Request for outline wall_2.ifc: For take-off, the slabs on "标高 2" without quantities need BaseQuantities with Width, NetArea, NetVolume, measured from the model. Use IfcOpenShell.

First a look at what the model holds.

```python
import ifcopenshell
import ifcopenshell.util.element
import ifcopenshell.util.unit

model = ifcopenshell.open("outline wall_2.ifc")
print(model.schema)
for unit_type in ("LENGTHUNIT", "AREAUNIT", "VOLUMEUNIT"):
    print(unit_type, ifcopenshell.util.unit.calculate_unit_scale(model, unit_type))
storey = next(s for s in model.by_type("IfcBuildingStorey") if s.Name == "标高 2")
slabs = [e for e in ifcopenshell.util.element.get_decomposition(storey) if e.is_a("IfcSlab")]
for e in sorted(slabs, key=lambda e: e.id()):
    print(e.id(), e.is_a(), e.Name, list(ifcopenshell.util.element.get_psets(e, qtos_only=True)), sep=" | ")
```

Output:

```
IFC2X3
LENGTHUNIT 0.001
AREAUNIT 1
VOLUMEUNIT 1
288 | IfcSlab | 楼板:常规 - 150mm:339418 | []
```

```python
import ifcopenshell
import ifcopenshell.api.pset
import ifcopenshell.geom
import ifcopenshell.util.element
import ifcopenshell.util.shape
import ifcopenshell.util.unit

model = ifcopenshell.open("outline wall_2.ifc")
unit_scale = ifcopenshell.util.unit.calculate_unit_scale(model)
area_scale = ifcopenshell.util.unit.calculate_unit_scale(model, "AREAUNIT")
volume_scale = ifcopenshell.util.unit.calculate_unit_scale(model, "VOLUMEUNIT")
settings = ifcopenshell.geom.settings()

storey = next(s for s in model.by_type("IfcBuildingStorey") if s.Name == "标高 2")
slabs = [e for e in ifcopenshell.util.element.get_decomposition(storey) if e.is_a("IfcSlab")]

for e in sorted(slabs, key=lambda e: e.id()):
    if ifcopenshell.util.element.get_psets(e, qtos_only=True, should_inherit=False):
        continue
    # Geometry comes back in metres, in the element's own axes.
    shape = ifcopenshell.geom.create_shape(settings, e)
    values = {
        "Width": ifcopenshell.util.shape.get_z(shape.geometry) / unit_scale,
        "NetArea": ifcopenshell.util.shape.get_footprint_area(shape.geometry) / area_scale,
        "NetVolume": ifcopenshell.util.shape.get_volume(shape.geometry) / volume_scale,
    }
    qto = ifcopenshell.api.pset.add_qto(model, product=e, name="BaseQuantities")
    ifcopenshell.api.pset.edit_qto(model, qto=qto, properties=values)
    print(e.id(), {k: round(v, 3) for k, v in values.items()})

model.write("outline wall_2_v2.ifc")
```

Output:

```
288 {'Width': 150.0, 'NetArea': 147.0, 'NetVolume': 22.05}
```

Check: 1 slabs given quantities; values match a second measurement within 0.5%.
